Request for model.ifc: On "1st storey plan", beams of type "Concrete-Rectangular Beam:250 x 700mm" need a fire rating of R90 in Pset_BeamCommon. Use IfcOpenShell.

First a look at what the model holds.

```python
import ifcopenshell
import ifcopenshell.util.element

model = ifcopenshell.open("model.ifc")
print(model.schema)
storey = next(s for s in model.by_type("IfcBuildingStorey") if s.Name == "1st storey plan")
beams = [e for e in ifcopenshell.util.element.get_decomposition(storey) if e.is_a("IfcBeam")]
seen = {}
for e in beams:
    element_type = ifcopenshell.util.element.get_type(e)
    key = (element_type.Name if element_type != e and element_type else None, ifcopenshell.util.element.get_pset(e, "Pset_BeamCommon", "FireRating"))
    seen[key] = seen.get(key, 0) + 1
for (name, value), count in sorted(seen.items(), key=str):
    print(count, "x", name, "|", value)
```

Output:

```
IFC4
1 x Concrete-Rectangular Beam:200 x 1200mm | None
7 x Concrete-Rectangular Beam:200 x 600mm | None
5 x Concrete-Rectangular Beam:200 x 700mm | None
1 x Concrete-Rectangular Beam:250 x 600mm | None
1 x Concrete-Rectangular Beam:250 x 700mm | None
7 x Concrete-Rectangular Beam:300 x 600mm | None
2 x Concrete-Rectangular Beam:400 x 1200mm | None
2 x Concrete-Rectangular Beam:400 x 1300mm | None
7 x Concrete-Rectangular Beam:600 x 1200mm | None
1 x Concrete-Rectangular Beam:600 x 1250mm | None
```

```python
import ifcopenshell
import ifcopenshell.api.pset
import ifcopenshell.util.element

model = ifcopenshell.open("model.ifc")

storey = next(s for s in model.by_type("IfcBuildingStorey") if s.Name == "1st storey plan")
beams = [e for e in ifcopenshell.util.element.get_decomposition(storey) if e.is_a("IfcBeam")]

count = 0
for e in beams:
    element_type = ifcopenshell.util.element.get_type(e)
    if element_type in (None, e) or element_type.Name != "Concrete-Rectangular Beam:250 x 700mm":
        continue
    # add_pset returns the element's existing set when there is one.
    pset = ifcopenshell.api.pset.add_pset(model, product=e, name="Pset_BeamCommon")
    ifcopenshell.api.pset.edit_pset(model, pset=pset, properties={"FireRating": "R90"})
    count += 1

print(count, "beams updated")

model.write("model_edited.ifc")
```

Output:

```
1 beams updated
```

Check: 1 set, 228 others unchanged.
